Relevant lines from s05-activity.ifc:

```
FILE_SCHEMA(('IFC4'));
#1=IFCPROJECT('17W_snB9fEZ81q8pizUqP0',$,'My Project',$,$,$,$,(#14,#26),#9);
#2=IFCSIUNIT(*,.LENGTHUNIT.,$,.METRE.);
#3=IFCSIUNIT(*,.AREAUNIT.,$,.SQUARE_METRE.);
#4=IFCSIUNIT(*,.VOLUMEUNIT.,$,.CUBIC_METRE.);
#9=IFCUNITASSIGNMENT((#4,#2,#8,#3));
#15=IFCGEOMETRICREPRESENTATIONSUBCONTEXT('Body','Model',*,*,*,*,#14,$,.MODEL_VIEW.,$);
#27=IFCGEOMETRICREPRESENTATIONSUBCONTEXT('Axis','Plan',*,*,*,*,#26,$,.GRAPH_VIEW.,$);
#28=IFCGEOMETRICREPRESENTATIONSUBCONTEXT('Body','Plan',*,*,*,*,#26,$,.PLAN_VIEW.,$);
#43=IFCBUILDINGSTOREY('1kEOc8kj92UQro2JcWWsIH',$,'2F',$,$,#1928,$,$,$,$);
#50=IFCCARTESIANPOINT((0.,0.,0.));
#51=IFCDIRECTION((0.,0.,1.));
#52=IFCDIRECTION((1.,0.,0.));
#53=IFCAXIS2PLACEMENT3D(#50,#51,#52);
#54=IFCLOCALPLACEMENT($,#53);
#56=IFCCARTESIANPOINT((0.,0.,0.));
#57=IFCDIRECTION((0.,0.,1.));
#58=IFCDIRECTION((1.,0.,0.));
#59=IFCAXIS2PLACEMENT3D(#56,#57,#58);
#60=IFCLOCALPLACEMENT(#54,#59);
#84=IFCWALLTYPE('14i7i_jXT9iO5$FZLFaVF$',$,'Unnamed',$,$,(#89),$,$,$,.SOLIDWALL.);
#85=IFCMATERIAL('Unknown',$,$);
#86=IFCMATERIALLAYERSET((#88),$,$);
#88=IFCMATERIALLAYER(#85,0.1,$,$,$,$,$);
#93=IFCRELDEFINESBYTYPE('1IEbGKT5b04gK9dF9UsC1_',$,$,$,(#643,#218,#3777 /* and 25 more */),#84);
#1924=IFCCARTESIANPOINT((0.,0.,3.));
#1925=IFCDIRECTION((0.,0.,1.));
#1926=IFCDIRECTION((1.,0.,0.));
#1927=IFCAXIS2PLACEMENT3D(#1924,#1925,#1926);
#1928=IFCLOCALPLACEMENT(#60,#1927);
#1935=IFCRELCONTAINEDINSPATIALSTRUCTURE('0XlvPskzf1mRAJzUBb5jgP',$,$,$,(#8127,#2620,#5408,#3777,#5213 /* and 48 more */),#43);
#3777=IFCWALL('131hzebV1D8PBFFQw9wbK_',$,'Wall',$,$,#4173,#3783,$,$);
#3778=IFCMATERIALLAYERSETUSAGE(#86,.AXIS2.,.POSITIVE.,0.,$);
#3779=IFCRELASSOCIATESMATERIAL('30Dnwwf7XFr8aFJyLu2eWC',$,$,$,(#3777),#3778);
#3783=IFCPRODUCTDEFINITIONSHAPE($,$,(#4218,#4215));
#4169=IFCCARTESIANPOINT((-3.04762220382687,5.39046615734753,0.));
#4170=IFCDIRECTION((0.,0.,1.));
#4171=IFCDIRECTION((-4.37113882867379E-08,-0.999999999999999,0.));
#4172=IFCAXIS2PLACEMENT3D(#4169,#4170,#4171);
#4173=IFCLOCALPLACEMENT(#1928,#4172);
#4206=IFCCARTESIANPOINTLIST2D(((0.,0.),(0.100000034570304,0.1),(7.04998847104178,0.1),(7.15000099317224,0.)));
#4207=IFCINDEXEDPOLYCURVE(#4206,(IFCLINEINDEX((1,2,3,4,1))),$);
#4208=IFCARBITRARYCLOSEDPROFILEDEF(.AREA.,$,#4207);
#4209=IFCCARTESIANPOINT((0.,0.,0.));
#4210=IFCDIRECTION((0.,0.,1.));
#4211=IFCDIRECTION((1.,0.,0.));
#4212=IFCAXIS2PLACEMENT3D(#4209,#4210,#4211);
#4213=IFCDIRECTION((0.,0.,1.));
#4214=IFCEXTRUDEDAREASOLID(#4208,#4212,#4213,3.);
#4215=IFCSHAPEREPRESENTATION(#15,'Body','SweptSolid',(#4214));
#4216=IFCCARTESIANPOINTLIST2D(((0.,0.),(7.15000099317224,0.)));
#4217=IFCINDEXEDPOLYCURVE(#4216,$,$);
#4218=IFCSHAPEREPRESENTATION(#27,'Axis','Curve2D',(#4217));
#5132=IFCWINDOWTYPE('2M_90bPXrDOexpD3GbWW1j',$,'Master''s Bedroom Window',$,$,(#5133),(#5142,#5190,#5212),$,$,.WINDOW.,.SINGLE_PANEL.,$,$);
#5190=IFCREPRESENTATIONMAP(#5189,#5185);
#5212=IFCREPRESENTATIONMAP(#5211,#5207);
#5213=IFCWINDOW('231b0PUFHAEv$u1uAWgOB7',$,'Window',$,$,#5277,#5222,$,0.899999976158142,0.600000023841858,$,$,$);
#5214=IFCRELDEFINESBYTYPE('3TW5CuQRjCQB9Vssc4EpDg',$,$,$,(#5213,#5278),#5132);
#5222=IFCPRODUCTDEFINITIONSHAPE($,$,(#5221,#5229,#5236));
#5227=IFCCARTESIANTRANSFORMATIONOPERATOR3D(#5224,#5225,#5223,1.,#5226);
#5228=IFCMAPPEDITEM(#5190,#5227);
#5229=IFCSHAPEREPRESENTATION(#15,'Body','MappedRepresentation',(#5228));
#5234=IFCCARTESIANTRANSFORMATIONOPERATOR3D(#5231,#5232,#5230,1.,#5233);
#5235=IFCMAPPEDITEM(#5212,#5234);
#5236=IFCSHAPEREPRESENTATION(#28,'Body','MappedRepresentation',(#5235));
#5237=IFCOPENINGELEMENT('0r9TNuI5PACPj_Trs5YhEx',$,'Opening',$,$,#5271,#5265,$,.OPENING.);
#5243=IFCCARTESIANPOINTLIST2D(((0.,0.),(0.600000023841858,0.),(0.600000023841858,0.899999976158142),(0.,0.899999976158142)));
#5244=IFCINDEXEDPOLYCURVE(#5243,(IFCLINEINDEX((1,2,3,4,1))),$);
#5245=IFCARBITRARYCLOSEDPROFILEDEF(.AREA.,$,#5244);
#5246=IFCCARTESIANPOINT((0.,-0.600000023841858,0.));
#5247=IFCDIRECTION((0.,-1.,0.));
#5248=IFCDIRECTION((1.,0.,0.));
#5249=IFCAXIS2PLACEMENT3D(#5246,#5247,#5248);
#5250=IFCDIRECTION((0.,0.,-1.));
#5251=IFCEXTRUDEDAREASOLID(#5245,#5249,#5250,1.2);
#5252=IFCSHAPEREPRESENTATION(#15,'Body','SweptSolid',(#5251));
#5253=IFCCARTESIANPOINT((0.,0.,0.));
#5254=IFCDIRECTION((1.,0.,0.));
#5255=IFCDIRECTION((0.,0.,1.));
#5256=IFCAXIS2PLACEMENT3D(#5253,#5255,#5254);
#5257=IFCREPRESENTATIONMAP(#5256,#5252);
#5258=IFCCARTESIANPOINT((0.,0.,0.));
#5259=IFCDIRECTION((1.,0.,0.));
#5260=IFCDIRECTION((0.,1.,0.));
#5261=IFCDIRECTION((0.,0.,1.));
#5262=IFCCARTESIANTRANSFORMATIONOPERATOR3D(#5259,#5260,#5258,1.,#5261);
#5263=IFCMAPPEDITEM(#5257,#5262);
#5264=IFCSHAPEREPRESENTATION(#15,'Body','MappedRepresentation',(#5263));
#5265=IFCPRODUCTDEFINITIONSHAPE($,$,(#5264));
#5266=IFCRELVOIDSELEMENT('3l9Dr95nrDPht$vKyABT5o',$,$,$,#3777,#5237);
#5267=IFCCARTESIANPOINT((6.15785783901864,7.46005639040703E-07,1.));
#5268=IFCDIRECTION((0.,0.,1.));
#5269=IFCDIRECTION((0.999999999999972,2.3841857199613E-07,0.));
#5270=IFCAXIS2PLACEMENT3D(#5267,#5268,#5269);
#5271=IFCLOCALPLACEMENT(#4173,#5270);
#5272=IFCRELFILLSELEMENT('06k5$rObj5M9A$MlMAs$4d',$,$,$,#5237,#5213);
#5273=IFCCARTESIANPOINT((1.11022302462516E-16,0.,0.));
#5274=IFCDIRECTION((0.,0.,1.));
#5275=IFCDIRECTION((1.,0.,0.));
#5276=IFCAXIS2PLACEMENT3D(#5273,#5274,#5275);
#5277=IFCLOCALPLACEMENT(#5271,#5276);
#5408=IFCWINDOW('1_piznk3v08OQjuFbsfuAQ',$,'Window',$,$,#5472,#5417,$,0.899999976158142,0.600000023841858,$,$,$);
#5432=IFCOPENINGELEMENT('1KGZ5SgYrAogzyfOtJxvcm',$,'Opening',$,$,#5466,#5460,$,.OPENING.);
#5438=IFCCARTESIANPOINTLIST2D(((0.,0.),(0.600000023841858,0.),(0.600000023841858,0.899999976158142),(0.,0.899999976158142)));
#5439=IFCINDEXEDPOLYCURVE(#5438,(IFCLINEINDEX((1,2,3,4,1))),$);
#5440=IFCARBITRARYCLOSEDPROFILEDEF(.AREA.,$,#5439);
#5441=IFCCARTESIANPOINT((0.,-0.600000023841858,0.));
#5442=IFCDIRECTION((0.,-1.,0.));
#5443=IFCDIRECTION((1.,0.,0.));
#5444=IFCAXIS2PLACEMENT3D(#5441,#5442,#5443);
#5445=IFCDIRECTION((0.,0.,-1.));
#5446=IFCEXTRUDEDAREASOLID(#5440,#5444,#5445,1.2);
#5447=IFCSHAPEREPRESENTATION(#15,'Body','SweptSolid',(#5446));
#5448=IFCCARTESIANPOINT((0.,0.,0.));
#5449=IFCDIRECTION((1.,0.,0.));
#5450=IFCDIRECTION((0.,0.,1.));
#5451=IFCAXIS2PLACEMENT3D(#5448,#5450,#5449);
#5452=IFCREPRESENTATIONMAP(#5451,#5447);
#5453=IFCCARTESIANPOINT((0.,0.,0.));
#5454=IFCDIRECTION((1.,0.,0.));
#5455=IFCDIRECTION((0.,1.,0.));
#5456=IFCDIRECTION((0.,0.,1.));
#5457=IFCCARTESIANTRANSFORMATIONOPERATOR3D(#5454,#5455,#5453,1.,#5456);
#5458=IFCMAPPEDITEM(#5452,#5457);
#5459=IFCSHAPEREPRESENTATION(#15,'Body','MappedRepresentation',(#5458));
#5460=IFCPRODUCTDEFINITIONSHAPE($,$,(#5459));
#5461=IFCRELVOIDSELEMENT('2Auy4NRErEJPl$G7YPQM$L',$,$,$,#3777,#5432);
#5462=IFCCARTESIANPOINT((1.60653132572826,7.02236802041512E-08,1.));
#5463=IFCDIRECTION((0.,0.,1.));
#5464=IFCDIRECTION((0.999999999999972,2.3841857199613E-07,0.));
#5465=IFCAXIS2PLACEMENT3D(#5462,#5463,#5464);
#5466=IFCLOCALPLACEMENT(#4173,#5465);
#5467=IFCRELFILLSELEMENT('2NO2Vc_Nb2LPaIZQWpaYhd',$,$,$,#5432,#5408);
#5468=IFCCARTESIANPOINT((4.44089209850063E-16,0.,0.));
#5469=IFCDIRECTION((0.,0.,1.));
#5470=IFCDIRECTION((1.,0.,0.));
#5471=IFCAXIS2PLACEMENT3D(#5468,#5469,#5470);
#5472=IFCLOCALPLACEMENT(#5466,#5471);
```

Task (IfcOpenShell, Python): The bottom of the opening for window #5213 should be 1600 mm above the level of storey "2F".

```python
import numpy as np
import ifcopenshell
import ifcopenshell.api.geometry
import ifcopenshell.geom
import ifcopenshell.util.element
import ifcopenshell.util.placement
import ifcopenshell.util.shape
import ifcopenshell.util.unit

model = ifcopenshell.open("s05-activity.ifc")
unit_scale = ifcopenshell.util.unit.calculate_unit_scale(model)

window = model.by_id(5213)
opening = window.FillsVoids[0].RelatingOpeningElement
storey = ifcopenshell.util.element.get_container(window, ifc_class="IfcBuildingStorey")
level = ifcopenshell.util.placement.get_local_placement(storey.ObjectPlacement)[2, 3]

# The opening's origin need not be at the sill, so measure its lowest point.
shape = ifcopenshell.geom.create_shape(ifcopenshell.geom.settings(), opening)
bottom = ifcopenshell.util.shape.get_shape_bottom_elevation(shape, shape.geometry) / unit_scale
dz = level + 1.6 - bottom

shift = np.array([0.0, 0.0, dz])
# The window is placed relative to its opening, so it follows when the opening moves.
matrix = ifcopenshell.util.placement.get_local_placement(opening.ObjectPlacement)
matrix[:3, 3] += shift
ifcopenshell.api.geometry.edit_object_placement(
    model, product=opening, matrix=matrix, is_si=False, should_transform_children=True
)

print(f"moved by {dz * unit_scale:+.3f} m")

model.write("s05-activity_v2.ifc")
```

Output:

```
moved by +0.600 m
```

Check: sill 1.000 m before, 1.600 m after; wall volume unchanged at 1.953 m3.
